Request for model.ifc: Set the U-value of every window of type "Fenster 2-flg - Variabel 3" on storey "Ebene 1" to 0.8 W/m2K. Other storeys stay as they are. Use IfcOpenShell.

First a look at what the model holds.

```python
import ifcopenshell
import ifcopenshell.util.element

model = ifcopenshell.open("model.ifc")
print(model.schema)
storey = next(s for s in model.by_type("IfcBuildingStorey") if s.Name == "Ebene 1")
windows = [e for e in ifcopenshell.util.element.get_decomposition(storey) if e.is_a("IfcWindow")]
seen = {}
for e in windows:
    element_type = ifcopenshell.util.element.get_type(e)
    key = (element_type.Name if element_type != e and element_type else None, ifcopenshell.util.element.get_pset(e, "Pset_WindowCommon", "ThermalTransmittance"))
    seen[key] = seen.get(key, 0) + 1
for (name, value), count in sorted(seen.items(), key=str):
    print(count, "x", name, "|", value)
```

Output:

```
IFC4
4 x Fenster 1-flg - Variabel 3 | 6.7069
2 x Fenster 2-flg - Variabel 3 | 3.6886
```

```python
import ifcopenshell
import ifcopenshell.api.pset
import ifcopenshell.util.element

model = ifcopenshell.open("model.ifc")

storey = next(s for s in model.by_type("IfcBuildingStorey") if s.Name == "Ebene 1")
windows = [e for e in ifcopenshell.util.element.get_decomposition(storey) if e.is_a("IfcWindow")]

count = 0
for e in windows:
    element_type = ifcopenshell.util.element.get_type(e)
    if element_type in (None, e) or element_type.Name != "Fenster 2-flg - Variabel 3":
        continue
    # add_pset returns the element's existing set when there is one.
    pset = ifcopenshell.api.pset.add_pset(model, product=e, name="Pset_WindowCommon")
    ifcopenshell.api.pset.edit_pset(model, pset=pset, properties={"ThermalTransmittance": 0.8})
    count += 1

print(count, "windows updated")

model.write("model_v2.ifc")
```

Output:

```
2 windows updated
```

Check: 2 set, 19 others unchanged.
